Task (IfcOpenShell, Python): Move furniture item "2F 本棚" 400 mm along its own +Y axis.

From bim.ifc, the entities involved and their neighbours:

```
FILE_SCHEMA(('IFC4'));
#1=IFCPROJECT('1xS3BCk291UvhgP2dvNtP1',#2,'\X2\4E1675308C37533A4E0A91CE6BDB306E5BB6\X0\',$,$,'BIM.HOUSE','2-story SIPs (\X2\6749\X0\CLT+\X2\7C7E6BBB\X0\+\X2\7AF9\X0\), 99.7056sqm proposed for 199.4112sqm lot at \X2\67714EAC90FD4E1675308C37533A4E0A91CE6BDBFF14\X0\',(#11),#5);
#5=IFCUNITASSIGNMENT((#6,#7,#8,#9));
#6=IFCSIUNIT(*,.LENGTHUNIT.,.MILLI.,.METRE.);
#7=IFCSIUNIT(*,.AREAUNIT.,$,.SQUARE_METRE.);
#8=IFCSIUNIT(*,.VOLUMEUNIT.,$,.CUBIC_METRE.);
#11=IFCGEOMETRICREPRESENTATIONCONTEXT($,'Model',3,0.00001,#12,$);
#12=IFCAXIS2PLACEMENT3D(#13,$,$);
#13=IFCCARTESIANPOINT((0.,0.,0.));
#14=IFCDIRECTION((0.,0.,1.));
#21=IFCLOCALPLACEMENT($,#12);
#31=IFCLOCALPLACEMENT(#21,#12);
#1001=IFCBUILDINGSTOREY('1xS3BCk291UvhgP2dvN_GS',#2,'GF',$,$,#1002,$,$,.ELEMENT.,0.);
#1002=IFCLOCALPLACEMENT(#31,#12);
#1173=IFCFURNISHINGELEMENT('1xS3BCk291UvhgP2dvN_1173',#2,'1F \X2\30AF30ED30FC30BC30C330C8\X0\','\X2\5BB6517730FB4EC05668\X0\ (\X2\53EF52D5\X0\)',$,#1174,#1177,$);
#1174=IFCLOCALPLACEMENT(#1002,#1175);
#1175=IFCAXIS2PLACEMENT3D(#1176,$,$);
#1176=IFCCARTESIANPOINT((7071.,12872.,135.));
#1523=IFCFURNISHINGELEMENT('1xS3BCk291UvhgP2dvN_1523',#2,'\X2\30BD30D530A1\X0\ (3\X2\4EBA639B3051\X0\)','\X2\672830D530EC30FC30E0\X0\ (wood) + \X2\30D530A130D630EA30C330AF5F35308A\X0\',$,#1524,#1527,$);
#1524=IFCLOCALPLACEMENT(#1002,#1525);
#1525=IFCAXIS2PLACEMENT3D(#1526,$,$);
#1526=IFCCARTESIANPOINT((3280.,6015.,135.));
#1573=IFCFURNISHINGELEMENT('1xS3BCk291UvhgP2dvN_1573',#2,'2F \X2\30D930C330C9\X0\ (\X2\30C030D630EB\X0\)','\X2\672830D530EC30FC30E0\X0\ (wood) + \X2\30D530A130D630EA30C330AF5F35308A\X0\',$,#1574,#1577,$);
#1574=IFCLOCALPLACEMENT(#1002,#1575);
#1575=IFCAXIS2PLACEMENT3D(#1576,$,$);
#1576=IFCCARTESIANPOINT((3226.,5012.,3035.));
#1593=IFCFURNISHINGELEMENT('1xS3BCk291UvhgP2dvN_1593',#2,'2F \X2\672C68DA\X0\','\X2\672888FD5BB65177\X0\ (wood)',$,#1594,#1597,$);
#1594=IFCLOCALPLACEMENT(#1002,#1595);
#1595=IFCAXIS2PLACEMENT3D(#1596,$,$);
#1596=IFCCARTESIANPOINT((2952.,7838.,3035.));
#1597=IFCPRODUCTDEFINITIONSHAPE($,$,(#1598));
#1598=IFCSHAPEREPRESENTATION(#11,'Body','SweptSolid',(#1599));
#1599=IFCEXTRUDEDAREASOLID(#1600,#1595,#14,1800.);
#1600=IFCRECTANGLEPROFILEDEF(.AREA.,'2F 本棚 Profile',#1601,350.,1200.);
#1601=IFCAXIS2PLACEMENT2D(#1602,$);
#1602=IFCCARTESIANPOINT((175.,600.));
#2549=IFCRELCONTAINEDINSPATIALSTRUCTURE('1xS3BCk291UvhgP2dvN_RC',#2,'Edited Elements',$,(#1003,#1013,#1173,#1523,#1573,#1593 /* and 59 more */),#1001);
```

```python
import ifcopenshell
import ifcopenshell.api.geometry
import ifcopenshell.util.placement
import ifcopenshell.util.unit

model = ifcopenshell.open("bim.ifc")
unit_scale = ifcopenshell.util.unit.calculate_unit_scale(model)

item = model.by_id(1593)
matrix = ifcopenshell.util.placement.get_local_placement(item.ObjectPlacement)
matrix[:3, 3] += matrix[:3, 1] * 0.4 / unit_scale
ifcopenshell.api.geometry.edit_object_placement(model, product=item, matrix=matrix, is_si=False)

print(ifcopenshell.util.placement.get_local_placement(item.ObjectPlacement).round(3) + 0.0)

model.write("bim_edited.ifc")
```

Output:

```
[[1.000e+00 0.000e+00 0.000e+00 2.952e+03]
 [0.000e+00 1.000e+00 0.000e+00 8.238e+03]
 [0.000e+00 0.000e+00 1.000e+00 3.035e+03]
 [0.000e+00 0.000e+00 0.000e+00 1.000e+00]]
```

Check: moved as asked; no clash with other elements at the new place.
